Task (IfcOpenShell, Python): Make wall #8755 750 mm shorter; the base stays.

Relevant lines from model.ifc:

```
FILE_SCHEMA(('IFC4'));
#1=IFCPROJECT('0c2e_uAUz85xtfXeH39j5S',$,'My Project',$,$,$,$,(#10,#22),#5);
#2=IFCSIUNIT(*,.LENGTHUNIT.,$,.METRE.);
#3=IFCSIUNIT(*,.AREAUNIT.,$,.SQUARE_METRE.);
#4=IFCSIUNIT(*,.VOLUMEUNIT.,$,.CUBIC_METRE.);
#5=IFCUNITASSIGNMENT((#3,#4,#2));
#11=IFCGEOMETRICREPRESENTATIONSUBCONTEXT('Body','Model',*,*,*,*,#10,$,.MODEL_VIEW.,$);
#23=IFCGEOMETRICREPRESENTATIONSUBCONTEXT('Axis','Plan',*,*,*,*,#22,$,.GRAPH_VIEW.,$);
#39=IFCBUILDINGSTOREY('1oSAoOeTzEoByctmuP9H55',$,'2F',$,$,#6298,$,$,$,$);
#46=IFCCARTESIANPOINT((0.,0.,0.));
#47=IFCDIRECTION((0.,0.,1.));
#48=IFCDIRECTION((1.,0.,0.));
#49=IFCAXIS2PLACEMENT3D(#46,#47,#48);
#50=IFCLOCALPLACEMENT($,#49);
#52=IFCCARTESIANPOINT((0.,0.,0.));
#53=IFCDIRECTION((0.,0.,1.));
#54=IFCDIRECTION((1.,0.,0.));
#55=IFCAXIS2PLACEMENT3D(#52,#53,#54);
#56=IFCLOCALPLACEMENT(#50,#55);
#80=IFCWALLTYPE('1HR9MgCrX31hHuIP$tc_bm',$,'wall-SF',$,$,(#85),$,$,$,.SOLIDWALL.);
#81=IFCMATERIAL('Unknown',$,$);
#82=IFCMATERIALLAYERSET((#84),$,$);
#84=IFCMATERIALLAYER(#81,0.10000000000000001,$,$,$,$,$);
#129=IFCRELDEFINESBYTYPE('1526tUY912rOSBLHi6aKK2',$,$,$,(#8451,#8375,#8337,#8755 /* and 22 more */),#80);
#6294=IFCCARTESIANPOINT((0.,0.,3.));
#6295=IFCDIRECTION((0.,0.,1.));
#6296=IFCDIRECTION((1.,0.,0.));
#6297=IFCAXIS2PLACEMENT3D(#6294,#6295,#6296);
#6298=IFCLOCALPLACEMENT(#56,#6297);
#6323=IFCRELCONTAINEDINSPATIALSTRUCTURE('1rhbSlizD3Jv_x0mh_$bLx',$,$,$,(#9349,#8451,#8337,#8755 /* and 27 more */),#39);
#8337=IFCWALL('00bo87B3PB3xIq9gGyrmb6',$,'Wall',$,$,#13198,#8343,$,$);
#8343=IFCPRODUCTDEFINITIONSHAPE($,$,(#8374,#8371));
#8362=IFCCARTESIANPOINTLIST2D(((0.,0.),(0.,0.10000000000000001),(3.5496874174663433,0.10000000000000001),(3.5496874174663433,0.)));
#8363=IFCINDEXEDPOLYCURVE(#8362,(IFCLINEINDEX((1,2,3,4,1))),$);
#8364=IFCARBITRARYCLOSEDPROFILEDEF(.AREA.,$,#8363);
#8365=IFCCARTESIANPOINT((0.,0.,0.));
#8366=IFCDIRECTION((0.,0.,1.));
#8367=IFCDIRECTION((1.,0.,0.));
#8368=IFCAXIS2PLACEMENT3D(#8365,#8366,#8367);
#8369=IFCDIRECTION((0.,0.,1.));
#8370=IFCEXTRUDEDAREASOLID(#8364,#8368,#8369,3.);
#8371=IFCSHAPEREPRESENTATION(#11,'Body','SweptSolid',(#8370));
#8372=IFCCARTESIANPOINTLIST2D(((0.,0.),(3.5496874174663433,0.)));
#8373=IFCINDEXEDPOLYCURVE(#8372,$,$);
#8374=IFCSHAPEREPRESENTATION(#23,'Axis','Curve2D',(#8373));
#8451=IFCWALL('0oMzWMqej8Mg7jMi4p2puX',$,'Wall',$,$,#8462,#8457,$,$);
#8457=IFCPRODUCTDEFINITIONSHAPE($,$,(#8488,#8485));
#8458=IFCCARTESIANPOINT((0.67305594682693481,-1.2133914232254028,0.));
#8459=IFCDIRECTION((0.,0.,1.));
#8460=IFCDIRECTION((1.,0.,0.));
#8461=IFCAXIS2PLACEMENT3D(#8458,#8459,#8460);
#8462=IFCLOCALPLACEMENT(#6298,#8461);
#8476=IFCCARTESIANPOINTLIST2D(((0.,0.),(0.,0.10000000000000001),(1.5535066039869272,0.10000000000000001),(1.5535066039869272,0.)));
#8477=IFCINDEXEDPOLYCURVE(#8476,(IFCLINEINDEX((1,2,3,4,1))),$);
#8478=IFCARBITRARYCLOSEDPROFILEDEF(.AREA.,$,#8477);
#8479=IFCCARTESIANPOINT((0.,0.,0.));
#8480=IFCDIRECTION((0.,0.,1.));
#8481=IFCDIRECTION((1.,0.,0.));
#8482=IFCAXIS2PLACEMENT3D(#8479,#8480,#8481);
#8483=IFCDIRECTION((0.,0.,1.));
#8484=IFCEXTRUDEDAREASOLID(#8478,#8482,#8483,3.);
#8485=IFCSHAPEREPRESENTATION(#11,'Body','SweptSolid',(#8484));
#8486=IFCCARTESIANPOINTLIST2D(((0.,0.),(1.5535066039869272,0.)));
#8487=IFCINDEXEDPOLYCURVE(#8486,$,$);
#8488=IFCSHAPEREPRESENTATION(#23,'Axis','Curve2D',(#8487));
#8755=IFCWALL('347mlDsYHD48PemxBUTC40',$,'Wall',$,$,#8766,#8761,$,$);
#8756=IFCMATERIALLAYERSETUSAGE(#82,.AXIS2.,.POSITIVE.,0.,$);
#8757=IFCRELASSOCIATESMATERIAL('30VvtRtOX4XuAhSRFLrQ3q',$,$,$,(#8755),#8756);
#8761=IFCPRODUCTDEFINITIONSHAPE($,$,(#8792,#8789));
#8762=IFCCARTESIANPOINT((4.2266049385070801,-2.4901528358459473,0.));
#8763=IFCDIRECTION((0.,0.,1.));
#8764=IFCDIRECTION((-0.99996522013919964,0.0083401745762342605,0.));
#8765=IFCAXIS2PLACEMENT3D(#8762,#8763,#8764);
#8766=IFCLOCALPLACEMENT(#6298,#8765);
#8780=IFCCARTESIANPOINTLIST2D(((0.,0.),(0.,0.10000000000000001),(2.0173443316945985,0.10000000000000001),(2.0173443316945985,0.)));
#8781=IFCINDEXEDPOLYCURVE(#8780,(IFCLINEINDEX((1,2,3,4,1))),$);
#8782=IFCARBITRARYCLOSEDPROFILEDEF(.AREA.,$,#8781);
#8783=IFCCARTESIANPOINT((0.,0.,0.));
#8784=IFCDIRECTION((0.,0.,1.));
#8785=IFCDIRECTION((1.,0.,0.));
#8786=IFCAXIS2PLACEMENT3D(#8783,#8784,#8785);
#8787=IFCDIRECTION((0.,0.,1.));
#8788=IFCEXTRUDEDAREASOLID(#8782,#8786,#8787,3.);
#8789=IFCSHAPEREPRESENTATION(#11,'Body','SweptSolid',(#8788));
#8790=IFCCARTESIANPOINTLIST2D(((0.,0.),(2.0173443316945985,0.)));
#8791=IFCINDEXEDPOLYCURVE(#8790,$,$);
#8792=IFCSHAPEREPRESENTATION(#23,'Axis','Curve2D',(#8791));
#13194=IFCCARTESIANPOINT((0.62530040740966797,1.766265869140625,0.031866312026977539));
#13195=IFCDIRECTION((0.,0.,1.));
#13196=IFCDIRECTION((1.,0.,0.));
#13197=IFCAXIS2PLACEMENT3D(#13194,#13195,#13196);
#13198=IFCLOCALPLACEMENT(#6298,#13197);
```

```python
import ifcopenshell
import ifcopenshell.geom
import ifcopenshell.util.representation
import ifcopenshell.util.shape
import ifcopenshell.util.unit

model = ifcopenshell.open("model.ifc")
unit_scale = ifcopenshell.util.unit.calculate_unit_scale(model)
settings = ifcopenshell.geom.settings()


def volume(element):
    """Net volume in cubic metres, openings subtracted."""
    shape = ifcopenshell.geom.create_shape(settings, element)
    return ifcopenshell.util.shape.get_volume(shape.geometry)


wall = model.by_guid("347mlDsYHD48PemxBUTC40")
before = volume(wall)

body = ifcopenshell.util.representation.get_representation(wall, "Model", "Body")
solid = body.Items[0]
old_height = solid.Depth
solid.Depth -= 0.75 / unit_scale
after = volume(wall)

print(f"height {old_height:g} -> {solid.Depth:g}, volume {before:.3f} -> {after:.3f} m3")

model.write("model_rev.ifc")
```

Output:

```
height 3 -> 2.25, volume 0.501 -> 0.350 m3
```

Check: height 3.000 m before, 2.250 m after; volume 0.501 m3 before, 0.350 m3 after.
